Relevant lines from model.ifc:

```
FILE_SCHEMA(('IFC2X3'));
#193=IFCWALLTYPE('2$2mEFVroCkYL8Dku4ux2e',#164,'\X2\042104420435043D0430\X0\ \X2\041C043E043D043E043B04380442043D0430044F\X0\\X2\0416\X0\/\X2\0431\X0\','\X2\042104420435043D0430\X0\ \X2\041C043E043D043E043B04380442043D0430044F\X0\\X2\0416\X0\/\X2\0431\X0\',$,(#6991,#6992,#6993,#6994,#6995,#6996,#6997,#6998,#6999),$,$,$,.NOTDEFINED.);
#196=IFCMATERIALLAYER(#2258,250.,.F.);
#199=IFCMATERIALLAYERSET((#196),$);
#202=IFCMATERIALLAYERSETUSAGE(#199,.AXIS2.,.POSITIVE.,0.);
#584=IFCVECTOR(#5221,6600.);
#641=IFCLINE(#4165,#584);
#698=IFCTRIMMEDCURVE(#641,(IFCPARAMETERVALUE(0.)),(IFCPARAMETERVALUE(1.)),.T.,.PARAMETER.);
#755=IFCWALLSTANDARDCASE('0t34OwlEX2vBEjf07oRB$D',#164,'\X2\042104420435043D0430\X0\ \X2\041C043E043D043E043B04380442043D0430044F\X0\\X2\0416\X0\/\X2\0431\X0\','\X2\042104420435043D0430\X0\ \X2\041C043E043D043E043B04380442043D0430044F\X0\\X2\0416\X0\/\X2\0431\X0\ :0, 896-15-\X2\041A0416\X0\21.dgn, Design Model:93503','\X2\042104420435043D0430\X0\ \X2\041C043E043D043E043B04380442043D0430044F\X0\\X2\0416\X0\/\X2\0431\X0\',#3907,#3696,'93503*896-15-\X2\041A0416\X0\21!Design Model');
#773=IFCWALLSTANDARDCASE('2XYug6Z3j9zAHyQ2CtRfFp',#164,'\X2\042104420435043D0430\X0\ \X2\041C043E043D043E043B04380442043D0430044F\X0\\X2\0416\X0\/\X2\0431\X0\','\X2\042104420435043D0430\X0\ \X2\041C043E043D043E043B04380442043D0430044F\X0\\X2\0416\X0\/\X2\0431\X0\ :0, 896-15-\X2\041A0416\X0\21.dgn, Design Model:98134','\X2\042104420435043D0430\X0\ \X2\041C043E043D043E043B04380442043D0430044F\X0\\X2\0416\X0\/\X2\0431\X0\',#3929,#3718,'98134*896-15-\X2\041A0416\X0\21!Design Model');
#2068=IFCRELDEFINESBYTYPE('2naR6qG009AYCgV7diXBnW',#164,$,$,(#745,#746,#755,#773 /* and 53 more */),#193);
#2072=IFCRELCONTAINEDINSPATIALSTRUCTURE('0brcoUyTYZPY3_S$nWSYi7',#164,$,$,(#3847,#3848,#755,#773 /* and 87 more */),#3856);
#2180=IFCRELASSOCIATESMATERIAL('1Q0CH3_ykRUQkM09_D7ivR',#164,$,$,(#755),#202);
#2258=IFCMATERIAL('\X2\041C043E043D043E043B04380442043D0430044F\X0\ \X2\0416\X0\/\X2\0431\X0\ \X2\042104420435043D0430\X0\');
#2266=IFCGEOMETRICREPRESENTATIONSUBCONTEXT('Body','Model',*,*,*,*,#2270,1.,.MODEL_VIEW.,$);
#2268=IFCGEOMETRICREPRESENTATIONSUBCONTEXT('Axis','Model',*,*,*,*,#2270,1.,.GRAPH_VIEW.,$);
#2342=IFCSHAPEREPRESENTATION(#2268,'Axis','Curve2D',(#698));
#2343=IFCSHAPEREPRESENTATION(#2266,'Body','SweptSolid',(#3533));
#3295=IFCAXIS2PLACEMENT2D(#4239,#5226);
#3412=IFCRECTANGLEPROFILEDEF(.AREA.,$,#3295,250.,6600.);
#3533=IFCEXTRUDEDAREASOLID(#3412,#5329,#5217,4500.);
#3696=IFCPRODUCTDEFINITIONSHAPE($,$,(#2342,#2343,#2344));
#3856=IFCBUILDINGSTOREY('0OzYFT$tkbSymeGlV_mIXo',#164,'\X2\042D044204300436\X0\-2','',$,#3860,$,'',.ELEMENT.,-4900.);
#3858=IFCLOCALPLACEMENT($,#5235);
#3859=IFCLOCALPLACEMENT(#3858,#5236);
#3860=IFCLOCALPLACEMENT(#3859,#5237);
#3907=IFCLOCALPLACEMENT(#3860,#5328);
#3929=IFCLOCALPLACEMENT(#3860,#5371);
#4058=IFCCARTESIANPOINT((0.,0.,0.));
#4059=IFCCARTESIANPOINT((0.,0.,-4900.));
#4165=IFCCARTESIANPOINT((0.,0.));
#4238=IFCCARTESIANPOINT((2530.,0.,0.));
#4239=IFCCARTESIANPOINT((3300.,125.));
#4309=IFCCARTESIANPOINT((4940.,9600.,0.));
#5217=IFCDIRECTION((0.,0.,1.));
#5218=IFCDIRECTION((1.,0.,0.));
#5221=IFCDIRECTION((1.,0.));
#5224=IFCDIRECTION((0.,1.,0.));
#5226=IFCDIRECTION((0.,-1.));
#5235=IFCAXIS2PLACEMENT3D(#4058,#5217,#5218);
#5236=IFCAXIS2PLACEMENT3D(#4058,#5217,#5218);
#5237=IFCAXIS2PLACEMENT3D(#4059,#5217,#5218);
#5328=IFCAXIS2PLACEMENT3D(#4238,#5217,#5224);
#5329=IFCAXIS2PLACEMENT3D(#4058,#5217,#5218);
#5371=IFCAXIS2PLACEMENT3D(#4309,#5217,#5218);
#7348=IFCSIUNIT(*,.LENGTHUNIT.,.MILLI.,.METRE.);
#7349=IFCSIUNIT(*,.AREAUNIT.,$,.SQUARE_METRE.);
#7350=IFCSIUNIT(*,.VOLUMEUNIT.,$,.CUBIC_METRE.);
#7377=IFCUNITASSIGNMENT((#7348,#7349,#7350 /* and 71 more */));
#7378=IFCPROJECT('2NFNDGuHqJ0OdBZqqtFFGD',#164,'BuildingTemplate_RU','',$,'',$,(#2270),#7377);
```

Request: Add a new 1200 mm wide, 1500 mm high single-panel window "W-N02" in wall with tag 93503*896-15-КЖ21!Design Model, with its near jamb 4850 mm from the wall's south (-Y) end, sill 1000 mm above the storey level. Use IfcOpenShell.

```python
import numpy as np
import ifcopenshell
import ifcopenshell.api.feature
import ifcopenshell.api.geometry
import ifcopenshell.api.root
import ifcopenshell.api.spatial
import ifcopenshell.api.type
import ifcopenshell.geom
import ifcopenshell.util.element
import ifcopenshell.util.placement
import ifcopenshell.util.representation
import ifcopenshell.util.shape
import ifcopenshell.util.unit

model = ifcopenshell.open("model.ifc")
unit_scale = ifcopenshell.util.unit.calculate_unit_scale(model)
settings = ifcopenshell.geom.settings()


def volume(element):
    """Net volume in cubic metres, openings subtracted."""
    shape = ifcopenshell.geom.create_shape(settings, element)
    return ifcopenshell.util.shape.get_volume(shape.geometry)


wall = model.by_guid("0t34OwlEX2vBEjf07oRB$D")
storey = ifcopenshell.util.element.get_container(wall, ifc_class="IfcBuildingStorey")
context = ifcopenshell.util.representation.get_context(model, "Model", "Body", "MODEL_VIEW")
before = volume(wall)

width, height, from_end, sill = 1.2, 1.5, 4.85, 1  # metres

# The wall runs along its own X axis, and the end named is its -X end.
wall_shape = ifcopenshell.geom.create_shape(settings, wall)
x, y, z = ifcopenshell.util.shape.get_vertices(wall_shape.geometry).T
start = x.min() + from_end
face, thickness = float(y.min()), float(y.max() - y.min())
wall_matrix = ifcopenshell.util.placement.get_local_placement(wall.ObjectPlacement)
level = ifcopenshell.util.placement.get_local_placement(storey.ObjectPlacement)[2, 3]


def in_wall(x, y):
    """Placement at x, y metres in the wall's axes, at sill height."""
    matrix = wall_matrix.copy()
    matrix[:, 3] = wall_matrix @ np.array([x / unit_scale, y / unit_scale, 0.0, 1.0])
    matrix[2, 3] = level + sill / unit_scale
    return matrix


# Opening: a box that overshoots both wall faces by 50 mm.
opening = ifcopenshell.api.root.create_entity(model, ifc_class="IfcOpeningElement")
box = ifcopenshell.api.geometry.add_wall_representation(
    model, context=context, length=width, height=height, thickness=thickness + 0.1
)
ifcopenshell.api.geometry.assign_representation(model, product=opening, representation=box)
ifcopenshell.api.geometry.edit_object_placement(model, product=opening, matrix=in_wall(start, face - 0.05), is_si=False)
ifcopenshell.api.feature.add_feature(model, feature=opening, element=wall)

window = ifcopenshell.api.root.create_entity(model, ifc_class="IfcWindow", name="W-N02")
window.OverallWidth, window.OverallHeight = width / unit_scale, height / unit_scale
body = ifcopenshell.api.geometry.add_window_representation(
    model,
    context=context,
    overall_width=window.OverallWidth,
    overall_height=window.OverallHeight,
    partition_type="SINGLE_PANEL",
)
ifcopenshell.api.geometry.assign_representation(model, product=window, representation=body)
ifcopenshell.api.spatial.assign_container(model, products=[window], relating_structure=storey)
fills = ifcopenshell.api.feature.add_filling(model, opening=opening, element=window)
fills.OwnerHistory = window.OwnerHistory  # required in IFC2X3

# IFC2X3 keeps the operation on the window style.
style = ifcopenshell.api.root.create_entity(model, ifc_class="IfcWindowStyle", name="W-N02")
style.OperationType, style.ConstructionType = "SINGLE_PANEL", "NOTDEFINED"
style.ParameterTakesPrecedence = style.Sizeable = False
ifcopenshell.api.type.assign_type(model, related_objects=[window], relating_type=style)

# Centre the window in the wall's thickness.
ifcopenshell.api.geometry.edit_object_placement(model, product=window, matrix=in_wall(start, face), is_si=False)
window_shape = ifcopenshell.geom.create_shape(settings, window)
depth = ifcopenshell.util.shape.get_vertices(window_shape.geometry)[:, 1]
offset = face + thickness / 2 - (depth.min() + depth.max()) / 2
ifcopenshell.api.geometry.edit_object_placement(model, product=window, matrix=in_wall(start, offset), is_si=False)

after = volume(wall)

print(f"wall volume {before:.3f} -> {after:.3f} m3")

model.write("model_v2.ifc")
```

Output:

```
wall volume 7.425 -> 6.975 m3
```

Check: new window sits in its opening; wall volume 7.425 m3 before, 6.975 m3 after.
